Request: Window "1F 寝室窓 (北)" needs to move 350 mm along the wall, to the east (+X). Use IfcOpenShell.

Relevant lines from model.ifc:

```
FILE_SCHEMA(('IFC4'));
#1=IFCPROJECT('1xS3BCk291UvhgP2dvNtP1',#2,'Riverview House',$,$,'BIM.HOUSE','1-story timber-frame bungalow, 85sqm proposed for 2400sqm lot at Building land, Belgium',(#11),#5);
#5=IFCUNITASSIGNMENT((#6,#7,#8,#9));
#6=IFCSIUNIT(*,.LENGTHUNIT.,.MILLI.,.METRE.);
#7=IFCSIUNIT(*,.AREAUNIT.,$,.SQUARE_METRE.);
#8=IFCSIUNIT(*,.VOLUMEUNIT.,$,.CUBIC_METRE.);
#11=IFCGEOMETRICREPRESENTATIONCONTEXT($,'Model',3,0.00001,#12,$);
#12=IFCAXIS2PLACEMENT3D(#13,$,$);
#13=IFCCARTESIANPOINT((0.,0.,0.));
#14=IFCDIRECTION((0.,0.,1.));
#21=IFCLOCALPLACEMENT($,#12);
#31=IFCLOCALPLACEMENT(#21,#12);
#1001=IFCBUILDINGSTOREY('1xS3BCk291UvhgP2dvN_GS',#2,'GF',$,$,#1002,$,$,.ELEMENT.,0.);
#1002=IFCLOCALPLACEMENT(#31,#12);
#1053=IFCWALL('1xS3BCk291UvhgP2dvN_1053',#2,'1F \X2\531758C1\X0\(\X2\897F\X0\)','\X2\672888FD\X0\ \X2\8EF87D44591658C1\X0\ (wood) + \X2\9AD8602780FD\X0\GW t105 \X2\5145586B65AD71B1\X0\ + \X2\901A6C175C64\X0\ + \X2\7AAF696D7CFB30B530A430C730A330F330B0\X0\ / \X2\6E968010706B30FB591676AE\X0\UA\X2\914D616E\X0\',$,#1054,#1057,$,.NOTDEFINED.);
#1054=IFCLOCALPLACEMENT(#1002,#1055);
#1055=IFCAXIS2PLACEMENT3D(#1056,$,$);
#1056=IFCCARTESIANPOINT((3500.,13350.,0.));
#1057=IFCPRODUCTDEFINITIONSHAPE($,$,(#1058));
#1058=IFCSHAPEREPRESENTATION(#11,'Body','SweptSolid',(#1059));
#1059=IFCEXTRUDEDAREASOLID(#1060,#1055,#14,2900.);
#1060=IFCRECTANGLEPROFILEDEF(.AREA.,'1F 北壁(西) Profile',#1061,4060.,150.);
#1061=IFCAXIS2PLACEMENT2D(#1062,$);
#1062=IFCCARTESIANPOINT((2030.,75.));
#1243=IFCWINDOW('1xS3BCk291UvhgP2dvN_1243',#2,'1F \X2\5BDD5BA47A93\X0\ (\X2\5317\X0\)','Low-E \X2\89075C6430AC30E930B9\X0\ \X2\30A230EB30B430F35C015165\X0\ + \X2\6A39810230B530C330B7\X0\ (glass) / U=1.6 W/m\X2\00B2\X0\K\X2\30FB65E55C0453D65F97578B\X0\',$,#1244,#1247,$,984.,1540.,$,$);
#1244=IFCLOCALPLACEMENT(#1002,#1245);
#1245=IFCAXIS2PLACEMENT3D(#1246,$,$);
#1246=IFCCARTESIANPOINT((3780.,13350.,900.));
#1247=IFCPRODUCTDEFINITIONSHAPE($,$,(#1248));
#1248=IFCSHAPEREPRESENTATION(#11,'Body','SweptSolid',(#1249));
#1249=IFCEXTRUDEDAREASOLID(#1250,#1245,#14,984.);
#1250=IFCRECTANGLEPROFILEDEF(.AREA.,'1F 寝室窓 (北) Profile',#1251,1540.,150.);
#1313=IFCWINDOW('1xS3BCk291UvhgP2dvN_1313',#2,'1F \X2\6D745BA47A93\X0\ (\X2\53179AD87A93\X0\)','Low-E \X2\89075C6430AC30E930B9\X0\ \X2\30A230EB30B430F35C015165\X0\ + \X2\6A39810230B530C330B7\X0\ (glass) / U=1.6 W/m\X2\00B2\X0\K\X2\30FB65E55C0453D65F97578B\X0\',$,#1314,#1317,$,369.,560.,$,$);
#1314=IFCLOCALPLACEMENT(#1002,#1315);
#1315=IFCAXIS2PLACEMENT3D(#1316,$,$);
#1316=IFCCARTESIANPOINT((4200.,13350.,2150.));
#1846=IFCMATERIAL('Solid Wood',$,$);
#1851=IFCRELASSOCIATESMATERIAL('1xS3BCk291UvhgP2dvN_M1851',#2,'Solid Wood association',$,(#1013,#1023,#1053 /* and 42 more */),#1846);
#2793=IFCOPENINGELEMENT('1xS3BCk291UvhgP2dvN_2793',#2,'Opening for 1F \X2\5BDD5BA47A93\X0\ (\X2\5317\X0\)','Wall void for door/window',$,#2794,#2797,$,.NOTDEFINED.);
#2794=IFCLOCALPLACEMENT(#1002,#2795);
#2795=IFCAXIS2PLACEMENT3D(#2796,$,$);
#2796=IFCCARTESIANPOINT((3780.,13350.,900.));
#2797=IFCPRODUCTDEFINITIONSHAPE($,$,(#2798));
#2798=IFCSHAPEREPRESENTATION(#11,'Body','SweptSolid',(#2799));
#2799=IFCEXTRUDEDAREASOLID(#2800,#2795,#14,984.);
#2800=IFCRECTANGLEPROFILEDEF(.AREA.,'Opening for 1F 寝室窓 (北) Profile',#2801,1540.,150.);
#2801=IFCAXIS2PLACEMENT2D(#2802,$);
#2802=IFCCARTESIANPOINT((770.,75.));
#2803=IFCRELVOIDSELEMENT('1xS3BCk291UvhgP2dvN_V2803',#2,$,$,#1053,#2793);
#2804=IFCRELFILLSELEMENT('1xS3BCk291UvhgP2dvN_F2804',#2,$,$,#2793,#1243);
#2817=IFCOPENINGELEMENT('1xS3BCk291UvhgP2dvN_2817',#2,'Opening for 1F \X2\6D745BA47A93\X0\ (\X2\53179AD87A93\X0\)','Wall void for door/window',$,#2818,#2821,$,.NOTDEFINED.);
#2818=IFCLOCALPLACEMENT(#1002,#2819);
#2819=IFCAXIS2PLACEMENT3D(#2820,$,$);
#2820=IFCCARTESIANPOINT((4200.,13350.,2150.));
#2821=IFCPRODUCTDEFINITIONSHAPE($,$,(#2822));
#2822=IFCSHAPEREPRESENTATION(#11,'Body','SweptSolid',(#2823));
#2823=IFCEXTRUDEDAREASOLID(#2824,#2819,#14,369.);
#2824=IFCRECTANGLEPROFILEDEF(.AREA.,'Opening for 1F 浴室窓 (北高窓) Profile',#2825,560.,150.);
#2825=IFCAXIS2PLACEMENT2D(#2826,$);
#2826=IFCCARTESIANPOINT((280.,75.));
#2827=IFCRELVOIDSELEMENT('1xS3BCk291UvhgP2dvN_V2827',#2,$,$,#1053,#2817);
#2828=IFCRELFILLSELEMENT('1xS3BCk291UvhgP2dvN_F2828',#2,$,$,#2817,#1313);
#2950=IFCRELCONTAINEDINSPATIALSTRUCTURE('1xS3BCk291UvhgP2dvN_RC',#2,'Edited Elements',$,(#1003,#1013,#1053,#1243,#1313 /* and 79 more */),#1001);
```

```python
import ifcopenshell
import ifcopenshell.api.geometry
import ifcopenshell.util.placement
import ifcopenshell.util.unit

model = ifcopenshell.open("model.ifc")
unit_scale = ifcopenshell.util.unit.calculate_unit_scale(model)

window = model.by_guid("1xS3BCk291UvhgP2dvN_1243")
opening = window.FillsVoids[0].RelatingOpeningElement
wall = opening.VoidsElements[0].RelatingBuildingElement

wall_matrix = ifcopenshell.util.placement.get_local_placement(wall.ObjectPlacement)
shift = wall_matrix[:3, 0] * 0.35 / unit_scale
before = ifcopenshell.util.placement.get_local_placement(window.ObjectPlacement)[:3, 3].copy()

# The window is not placed relative to its opening, so move both.
for product in (opening, window):
    matrix = ifcopenshell.util.placement.get_local_placement(product.ObjectPlacement)
    matrix[:3, 3] += shift
    ifcopenshell.api.geometry.edit_object_placement(model, product=product, matrix=matrix, is_si=False)

after = ifcopenshell.util.placement.get_local_placement(window.ObjectPlacement)[:3, 3]
print("window moved by", (after - before).round(3) + 0.0)

model.write("model_updated.ifc")
```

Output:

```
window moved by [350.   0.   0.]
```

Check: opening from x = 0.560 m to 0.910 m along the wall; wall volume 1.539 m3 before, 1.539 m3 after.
